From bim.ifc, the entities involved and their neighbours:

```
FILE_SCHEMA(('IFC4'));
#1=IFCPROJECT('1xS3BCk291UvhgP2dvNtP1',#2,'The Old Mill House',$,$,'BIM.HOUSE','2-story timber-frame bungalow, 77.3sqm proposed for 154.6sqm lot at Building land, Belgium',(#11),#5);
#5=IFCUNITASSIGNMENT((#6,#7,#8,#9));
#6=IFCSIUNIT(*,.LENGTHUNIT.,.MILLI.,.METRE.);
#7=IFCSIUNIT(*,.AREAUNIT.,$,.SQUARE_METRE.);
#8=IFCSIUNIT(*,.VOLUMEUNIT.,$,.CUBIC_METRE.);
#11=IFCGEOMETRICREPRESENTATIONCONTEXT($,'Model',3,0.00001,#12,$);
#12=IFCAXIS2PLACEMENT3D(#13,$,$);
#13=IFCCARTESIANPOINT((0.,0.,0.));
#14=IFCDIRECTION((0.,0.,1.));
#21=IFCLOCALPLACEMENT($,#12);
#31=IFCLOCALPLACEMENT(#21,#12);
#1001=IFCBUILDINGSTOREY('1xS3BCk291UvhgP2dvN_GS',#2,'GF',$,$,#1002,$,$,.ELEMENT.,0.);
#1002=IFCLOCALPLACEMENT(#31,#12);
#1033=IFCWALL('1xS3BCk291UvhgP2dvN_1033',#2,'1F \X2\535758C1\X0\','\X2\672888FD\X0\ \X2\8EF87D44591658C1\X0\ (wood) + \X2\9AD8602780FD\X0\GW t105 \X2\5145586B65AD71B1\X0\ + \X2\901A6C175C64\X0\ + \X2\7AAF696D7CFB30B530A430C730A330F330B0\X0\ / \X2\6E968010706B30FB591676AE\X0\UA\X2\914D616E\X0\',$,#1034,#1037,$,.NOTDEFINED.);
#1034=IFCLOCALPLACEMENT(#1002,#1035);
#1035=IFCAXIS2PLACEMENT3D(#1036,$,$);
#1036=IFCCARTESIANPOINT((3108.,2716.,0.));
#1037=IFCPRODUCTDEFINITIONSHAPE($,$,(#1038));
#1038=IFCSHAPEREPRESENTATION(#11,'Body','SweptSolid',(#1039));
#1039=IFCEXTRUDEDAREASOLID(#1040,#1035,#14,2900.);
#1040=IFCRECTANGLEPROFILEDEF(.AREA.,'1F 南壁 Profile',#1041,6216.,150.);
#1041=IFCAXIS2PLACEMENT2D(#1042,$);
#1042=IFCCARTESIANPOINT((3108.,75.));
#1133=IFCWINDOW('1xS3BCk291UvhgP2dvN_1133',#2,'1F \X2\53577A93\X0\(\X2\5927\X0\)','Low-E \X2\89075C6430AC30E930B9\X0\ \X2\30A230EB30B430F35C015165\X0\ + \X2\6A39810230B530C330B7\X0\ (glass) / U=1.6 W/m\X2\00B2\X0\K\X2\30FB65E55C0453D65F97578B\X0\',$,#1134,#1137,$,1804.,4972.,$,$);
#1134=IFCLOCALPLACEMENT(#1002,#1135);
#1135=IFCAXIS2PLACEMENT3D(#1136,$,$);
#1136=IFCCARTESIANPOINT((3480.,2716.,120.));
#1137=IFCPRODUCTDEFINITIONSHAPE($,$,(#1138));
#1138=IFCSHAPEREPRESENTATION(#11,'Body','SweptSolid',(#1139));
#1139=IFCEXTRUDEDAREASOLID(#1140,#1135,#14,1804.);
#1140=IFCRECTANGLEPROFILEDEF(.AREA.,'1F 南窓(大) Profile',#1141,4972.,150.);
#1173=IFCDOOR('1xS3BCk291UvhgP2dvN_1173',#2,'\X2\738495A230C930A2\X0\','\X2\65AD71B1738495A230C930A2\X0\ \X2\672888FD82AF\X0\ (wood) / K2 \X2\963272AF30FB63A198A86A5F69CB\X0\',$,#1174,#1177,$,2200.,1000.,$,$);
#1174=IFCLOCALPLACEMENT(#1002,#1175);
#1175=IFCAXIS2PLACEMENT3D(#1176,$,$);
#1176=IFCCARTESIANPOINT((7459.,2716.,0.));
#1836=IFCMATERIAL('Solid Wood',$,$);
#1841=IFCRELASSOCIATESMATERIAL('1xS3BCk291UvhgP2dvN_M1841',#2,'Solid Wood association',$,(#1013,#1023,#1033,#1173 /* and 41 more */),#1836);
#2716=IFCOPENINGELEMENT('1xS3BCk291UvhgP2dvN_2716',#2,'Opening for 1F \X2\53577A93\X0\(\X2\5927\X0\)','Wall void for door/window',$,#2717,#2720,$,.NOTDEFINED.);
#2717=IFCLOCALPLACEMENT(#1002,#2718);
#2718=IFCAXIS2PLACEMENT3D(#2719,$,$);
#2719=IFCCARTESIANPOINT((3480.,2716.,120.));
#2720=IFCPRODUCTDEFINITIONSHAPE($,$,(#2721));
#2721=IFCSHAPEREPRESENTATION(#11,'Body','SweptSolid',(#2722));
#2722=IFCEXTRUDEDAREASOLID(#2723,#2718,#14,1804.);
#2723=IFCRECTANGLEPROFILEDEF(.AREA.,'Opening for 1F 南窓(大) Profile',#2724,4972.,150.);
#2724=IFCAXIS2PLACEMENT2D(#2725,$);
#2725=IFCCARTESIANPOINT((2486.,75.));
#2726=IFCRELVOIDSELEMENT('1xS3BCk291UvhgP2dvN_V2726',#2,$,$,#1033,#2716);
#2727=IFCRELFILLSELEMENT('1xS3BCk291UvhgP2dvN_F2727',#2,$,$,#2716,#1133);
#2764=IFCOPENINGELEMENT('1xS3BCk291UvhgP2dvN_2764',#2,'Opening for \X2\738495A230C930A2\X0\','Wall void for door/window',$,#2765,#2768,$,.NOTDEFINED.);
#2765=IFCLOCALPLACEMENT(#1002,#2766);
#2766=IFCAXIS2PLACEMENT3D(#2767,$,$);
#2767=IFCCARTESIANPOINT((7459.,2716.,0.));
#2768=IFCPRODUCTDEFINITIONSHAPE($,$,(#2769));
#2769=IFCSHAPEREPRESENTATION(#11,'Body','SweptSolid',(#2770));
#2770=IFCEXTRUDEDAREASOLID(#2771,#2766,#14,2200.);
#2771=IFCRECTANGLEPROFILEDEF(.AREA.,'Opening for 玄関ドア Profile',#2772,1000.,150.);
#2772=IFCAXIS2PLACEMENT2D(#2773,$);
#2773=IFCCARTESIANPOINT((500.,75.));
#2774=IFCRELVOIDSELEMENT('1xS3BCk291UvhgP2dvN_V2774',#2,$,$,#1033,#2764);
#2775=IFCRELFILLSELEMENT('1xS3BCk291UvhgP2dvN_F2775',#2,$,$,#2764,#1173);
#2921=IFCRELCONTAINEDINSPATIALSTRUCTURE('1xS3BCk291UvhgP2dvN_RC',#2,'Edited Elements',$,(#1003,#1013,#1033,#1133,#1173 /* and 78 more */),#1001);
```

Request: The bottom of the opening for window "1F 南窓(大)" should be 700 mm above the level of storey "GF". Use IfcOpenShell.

```python
import numpy as np
import ifcopenshell
import ifcopenshell.api.geometry
import ifcopenshell.geom
import ifcopenshell.util.element
import ifcopenshell.util.placement
import ifcopenshell.util.shape
import ifcopenshell.util.unit

model = ifcopenshell.open("bim.ifc")
unit_scale = ifcopenshell.util.unit.calculate_unit_scale(model)

window = model.by_guid("1xS3BCk291UvhgP2dvN_1133")
opening = window.FillsVoids[0].RelatingOpeningElement
storey = ifcopenshell.util.element.get_container(window, ifc_class="IfcBuildingStorey")
level = ifcopenshell.util.placement.get_local_placement(storey.ObjectPlacement)[2, 3]

# The opening's origin need not be at the sill, so measure its lowest point.
shape = ifcopenshell.geom.create_shape(ifcopenshell.geom.settings(), opening)
bottom = ifcopenshell.util.shape.get_shape_bottom_elevation(shape, shape.geometry) / unit_scale
dz = level + 0.7 / unit_scale - bottom

shift = np.array([0.0, 0.0, dz])
# The window is not placed relative to its opening, so move both.
for product in (opening, window):
    matrix = ifcopenshell.util.placement.get_local_placement(product.ObjectPlacement)
    matrix[:3, 3] += shift
    ifcopenshell.api.geometry.edit_object_placement(model, product=product, matrix=matrix, is_si=False)

print(f"moved by {dz * unit_scale:+.3f} m")

model.write("bim-out.ifc")
```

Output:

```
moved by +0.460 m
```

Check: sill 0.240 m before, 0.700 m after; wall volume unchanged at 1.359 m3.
